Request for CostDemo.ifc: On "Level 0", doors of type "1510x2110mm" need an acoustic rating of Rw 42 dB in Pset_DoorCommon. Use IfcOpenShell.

First a look at what the model holds.

```python
import ifcopenshell
import ifcopenshell.util.element

model = ifcopenshell.open("CostDemo.ifc")
print(model.schema)
storey = next(s for s in model.by_type("IfcBuildingStorey") if s.Name == "Level 0")
doors = [e for e in ifcopenshell.util.element.get_decomposition(storey) if e.is_a("IfcDoor")]
seen = {}
for e in doors:
    element_type = ifcopenshell.util.element.get_type(e)
    key = (element_type.Name if element_type != e and element_type else None, ifcopenshell.util.element.get_pset(e, "Pset_DoorCommon", "AcousticRating"))
    seen[key] = seen.get(key, 0) + 1
for (name, value), count in sorted(seen.items(), key=str):
    print(count, "x", name, "|", value)
```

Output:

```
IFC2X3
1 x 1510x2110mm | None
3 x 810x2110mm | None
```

```python
import ifcopenshell
import ifcopenshell.api.pset
import ifcopenshell.util.element

model = ifcopenshell.open("CostDemo.ifc")

storey = next(s for s in model.by_type("IfcBuildingStorey") if s.Name == "Level 0")
doors = [e for e in ifcopenshell.util.element.get_decomposition(storey) if e.is_a("IfcDoor")]

count = 0
for e in doors:
    element_type = ifcopenshell.util.element.get_type(e)
    if element_type in (None, e) or element_type.Name != "1510x2110mm":
        continue
    # add_pset returns the element's existing set when there is one.
    pset = ifcopenshell.api.pset.add_pset(model, product=e, name="Pset_DoorCommon")
    ifcopenshell.api.pset.edit_pset(model, pset=pset, properties={"AcousticRating": "Rw 42 dB"})
    count += 1

print(count, "doors updated")

model.write("CostDemo_updated.ifc")
```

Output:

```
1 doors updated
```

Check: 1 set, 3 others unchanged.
